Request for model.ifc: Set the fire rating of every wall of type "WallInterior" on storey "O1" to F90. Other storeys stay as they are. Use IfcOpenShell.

First a look at what the model holds.

```python
import ifcopenshell
import ifcopenshell.util.element

model = ifcopenshell.open("model.ifc")
print(model.schema)
storey = next(s for s in model.by_type("IfcBuildingStorey") if s.Name == "O1")
walls = [e for e in ifcopenshell.util.element.get_decomposition(storey) if e.is_a("IfcWall")]
seen = {}
for e in walls:
    element_type = ifcopenshell.util.element.get_type(e)
    key = (element_type.Name if element_type != e and element_type else None, ifcopenshell.util.element.get_pset(e, "Pset_WallCommon", "FireRating"))
    seen[key] = seen.get(key, 0) + 1
for (name, value), count in sorted(seen.items(), key=str):
    print(count, "x", name, "|", value)
```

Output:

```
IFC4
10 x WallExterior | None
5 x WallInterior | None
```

```python
import ifcopenshell
import ifcopenshell.api.pset
import ifcopenshell.util.element

model = ifcopenshell.open("model.ifc")

storey = next(s for s in model.by_type("IfcBuildingStorey") if s.Name == "O1")
walls = [e for e in ifcopenshell.util.element.get_decomposition(storey) if e.is_a("IfcWall")]

count = 0
for e in walls:
    element_type = ifcopenshell.util.element.get_type(e)
    if element_type in (None, e) or element_type.Name != "WallInterior":
        continue
    # add_pset returns the element's existing set when there is one.
    pset = ifcopenshell.api.pset.add_pset(model, product=e, name="Pset_WallCommon")
    ifcopenshell.api.pset.edit_pset(model, pset=pset, properties={"FireRating": "F90"})
    count += 1

print(count, "walls updated")

model.write("model_rev.ifc")
```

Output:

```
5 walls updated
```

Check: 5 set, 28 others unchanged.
